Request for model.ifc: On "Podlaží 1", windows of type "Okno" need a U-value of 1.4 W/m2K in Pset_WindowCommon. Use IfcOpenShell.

First a look at what the model holds.

```python
import ifcopenshell
import ifcopenshell.util.element

model = ifcopenshell.open("model.ifc")
print(model.schema)
storey = next(s for s in model.by_type("IfcBuildingStorey") if s.Name == "Podlaží 1")
windows = [e for e in ifcopenshell.util.element.get_decomposition(storey) if e.is_a("IfcWindow")]
seen = {}
for e in windows:
    element_type = ifcopenshell.util.element.get_type(e)
    key = (element_type.Name if element_type != e and element_type else None, ifcopenshell.util.element.get_pset(e, "Pset_WindowCommon", "ThermalTransmittance"))
    seen[key] = seen.get(key, 0) + 1
for (name, value), count in sorted(seen.items(), key=str):
    print(count, "x", name, "|", value)
```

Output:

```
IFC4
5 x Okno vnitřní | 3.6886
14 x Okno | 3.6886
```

```python
import ifcopenshell
import ifcopenshell.api.pset
import ifcopenshell.util.element

model = ifcopenshell.open("model.ifc")

storey = next(s for s in model.by_type("IfcBuildingStorey") if s.Name == "Podlaží 1")
windows = [e for e in ifcopenshell.util.element.get_decomposition(storey) if e.is_a("IfcWindow")]

count = 0
for e in windows:
    element_type = ifcopenshell.util.element.get_type(e)
    if element_type in (None, e) or element_type.Name != "Okno":
        continue
    # add_pset returns the element's existing set when there is one.
    pset = ifcopenshell.api.pset.add_pset(model, product=e, name="Pset_WindowCommon")
    ifcopenshell.api.pset.edit_pset(model, pset=pset, properties={"ThermalTransmittance": 1.4})
    count += 1

print(count, "windows updated")

model.write("model_updated.ifc")
```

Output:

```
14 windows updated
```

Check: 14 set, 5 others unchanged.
